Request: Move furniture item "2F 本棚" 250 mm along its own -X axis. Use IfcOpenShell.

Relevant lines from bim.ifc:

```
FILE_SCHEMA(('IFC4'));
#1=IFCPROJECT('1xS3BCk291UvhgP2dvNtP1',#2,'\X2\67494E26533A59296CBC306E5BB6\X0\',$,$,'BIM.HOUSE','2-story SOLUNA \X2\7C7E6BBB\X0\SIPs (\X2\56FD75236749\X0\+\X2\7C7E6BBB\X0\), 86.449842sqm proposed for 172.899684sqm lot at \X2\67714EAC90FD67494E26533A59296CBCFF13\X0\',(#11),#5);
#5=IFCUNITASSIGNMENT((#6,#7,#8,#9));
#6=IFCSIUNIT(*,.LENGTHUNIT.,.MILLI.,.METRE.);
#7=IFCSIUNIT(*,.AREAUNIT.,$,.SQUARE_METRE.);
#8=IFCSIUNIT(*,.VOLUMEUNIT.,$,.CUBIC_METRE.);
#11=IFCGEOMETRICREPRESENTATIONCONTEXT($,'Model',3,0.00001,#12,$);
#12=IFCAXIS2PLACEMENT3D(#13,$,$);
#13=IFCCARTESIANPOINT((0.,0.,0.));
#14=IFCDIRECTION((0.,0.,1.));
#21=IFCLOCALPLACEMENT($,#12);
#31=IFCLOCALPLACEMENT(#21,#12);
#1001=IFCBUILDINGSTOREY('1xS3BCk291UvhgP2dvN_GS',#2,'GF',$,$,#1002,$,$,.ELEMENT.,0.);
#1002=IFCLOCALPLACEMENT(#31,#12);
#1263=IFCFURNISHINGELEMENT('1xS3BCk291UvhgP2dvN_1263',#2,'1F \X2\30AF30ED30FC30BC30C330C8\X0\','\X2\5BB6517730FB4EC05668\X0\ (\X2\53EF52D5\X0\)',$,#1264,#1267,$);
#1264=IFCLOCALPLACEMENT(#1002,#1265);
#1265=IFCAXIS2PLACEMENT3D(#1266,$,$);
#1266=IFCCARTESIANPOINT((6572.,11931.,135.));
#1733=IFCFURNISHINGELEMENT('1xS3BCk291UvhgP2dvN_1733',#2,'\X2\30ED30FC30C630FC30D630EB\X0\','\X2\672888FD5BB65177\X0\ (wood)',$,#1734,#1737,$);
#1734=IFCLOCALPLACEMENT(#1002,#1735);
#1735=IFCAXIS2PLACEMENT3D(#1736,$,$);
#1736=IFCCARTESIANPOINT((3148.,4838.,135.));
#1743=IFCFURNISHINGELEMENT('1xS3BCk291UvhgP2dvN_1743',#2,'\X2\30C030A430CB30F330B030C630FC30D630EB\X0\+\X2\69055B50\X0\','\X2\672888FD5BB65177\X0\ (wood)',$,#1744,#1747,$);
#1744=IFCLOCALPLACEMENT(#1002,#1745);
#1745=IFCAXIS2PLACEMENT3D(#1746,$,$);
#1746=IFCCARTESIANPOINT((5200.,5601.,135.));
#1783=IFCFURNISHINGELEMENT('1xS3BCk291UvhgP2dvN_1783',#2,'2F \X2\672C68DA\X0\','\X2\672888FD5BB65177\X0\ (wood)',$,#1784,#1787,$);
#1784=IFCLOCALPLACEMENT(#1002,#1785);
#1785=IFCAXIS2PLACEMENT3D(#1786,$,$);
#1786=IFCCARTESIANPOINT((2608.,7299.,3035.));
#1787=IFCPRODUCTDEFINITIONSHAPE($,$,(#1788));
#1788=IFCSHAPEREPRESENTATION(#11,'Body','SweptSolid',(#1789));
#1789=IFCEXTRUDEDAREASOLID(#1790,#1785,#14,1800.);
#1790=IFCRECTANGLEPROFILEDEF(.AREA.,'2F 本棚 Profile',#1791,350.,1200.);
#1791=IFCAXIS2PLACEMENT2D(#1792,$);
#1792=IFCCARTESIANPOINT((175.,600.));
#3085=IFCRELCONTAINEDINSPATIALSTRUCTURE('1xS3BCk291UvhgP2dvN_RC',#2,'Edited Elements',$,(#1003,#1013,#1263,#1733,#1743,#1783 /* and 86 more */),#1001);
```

```python
import ifcopenshell
import ifcopenshell.api.geometry
import ifcopenshell.util.placement

model = ifcopenshell.open("bim.ifc")

item = model.by_id(1783)
matrix = ifcopenshell.util.placement.get_local_placement(item.ObjectPlacement)
matrix[:3, 3] -= matrix[:3, 0] * 250.0
ifcopenshell.api.geometry.edit_object_placement(model, product=item, matrix=matrix, is_si=False)

print(ifcopenshell.util.placement.get_local_placement(item.ObjectPlacement).round(3) + 0.0)

model.write("bim-out.ifc")
```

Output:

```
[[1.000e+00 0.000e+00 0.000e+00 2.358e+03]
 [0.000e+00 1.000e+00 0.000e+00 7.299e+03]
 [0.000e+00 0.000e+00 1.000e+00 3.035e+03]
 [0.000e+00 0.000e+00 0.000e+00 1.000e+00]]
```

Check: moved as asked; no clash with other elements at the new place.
